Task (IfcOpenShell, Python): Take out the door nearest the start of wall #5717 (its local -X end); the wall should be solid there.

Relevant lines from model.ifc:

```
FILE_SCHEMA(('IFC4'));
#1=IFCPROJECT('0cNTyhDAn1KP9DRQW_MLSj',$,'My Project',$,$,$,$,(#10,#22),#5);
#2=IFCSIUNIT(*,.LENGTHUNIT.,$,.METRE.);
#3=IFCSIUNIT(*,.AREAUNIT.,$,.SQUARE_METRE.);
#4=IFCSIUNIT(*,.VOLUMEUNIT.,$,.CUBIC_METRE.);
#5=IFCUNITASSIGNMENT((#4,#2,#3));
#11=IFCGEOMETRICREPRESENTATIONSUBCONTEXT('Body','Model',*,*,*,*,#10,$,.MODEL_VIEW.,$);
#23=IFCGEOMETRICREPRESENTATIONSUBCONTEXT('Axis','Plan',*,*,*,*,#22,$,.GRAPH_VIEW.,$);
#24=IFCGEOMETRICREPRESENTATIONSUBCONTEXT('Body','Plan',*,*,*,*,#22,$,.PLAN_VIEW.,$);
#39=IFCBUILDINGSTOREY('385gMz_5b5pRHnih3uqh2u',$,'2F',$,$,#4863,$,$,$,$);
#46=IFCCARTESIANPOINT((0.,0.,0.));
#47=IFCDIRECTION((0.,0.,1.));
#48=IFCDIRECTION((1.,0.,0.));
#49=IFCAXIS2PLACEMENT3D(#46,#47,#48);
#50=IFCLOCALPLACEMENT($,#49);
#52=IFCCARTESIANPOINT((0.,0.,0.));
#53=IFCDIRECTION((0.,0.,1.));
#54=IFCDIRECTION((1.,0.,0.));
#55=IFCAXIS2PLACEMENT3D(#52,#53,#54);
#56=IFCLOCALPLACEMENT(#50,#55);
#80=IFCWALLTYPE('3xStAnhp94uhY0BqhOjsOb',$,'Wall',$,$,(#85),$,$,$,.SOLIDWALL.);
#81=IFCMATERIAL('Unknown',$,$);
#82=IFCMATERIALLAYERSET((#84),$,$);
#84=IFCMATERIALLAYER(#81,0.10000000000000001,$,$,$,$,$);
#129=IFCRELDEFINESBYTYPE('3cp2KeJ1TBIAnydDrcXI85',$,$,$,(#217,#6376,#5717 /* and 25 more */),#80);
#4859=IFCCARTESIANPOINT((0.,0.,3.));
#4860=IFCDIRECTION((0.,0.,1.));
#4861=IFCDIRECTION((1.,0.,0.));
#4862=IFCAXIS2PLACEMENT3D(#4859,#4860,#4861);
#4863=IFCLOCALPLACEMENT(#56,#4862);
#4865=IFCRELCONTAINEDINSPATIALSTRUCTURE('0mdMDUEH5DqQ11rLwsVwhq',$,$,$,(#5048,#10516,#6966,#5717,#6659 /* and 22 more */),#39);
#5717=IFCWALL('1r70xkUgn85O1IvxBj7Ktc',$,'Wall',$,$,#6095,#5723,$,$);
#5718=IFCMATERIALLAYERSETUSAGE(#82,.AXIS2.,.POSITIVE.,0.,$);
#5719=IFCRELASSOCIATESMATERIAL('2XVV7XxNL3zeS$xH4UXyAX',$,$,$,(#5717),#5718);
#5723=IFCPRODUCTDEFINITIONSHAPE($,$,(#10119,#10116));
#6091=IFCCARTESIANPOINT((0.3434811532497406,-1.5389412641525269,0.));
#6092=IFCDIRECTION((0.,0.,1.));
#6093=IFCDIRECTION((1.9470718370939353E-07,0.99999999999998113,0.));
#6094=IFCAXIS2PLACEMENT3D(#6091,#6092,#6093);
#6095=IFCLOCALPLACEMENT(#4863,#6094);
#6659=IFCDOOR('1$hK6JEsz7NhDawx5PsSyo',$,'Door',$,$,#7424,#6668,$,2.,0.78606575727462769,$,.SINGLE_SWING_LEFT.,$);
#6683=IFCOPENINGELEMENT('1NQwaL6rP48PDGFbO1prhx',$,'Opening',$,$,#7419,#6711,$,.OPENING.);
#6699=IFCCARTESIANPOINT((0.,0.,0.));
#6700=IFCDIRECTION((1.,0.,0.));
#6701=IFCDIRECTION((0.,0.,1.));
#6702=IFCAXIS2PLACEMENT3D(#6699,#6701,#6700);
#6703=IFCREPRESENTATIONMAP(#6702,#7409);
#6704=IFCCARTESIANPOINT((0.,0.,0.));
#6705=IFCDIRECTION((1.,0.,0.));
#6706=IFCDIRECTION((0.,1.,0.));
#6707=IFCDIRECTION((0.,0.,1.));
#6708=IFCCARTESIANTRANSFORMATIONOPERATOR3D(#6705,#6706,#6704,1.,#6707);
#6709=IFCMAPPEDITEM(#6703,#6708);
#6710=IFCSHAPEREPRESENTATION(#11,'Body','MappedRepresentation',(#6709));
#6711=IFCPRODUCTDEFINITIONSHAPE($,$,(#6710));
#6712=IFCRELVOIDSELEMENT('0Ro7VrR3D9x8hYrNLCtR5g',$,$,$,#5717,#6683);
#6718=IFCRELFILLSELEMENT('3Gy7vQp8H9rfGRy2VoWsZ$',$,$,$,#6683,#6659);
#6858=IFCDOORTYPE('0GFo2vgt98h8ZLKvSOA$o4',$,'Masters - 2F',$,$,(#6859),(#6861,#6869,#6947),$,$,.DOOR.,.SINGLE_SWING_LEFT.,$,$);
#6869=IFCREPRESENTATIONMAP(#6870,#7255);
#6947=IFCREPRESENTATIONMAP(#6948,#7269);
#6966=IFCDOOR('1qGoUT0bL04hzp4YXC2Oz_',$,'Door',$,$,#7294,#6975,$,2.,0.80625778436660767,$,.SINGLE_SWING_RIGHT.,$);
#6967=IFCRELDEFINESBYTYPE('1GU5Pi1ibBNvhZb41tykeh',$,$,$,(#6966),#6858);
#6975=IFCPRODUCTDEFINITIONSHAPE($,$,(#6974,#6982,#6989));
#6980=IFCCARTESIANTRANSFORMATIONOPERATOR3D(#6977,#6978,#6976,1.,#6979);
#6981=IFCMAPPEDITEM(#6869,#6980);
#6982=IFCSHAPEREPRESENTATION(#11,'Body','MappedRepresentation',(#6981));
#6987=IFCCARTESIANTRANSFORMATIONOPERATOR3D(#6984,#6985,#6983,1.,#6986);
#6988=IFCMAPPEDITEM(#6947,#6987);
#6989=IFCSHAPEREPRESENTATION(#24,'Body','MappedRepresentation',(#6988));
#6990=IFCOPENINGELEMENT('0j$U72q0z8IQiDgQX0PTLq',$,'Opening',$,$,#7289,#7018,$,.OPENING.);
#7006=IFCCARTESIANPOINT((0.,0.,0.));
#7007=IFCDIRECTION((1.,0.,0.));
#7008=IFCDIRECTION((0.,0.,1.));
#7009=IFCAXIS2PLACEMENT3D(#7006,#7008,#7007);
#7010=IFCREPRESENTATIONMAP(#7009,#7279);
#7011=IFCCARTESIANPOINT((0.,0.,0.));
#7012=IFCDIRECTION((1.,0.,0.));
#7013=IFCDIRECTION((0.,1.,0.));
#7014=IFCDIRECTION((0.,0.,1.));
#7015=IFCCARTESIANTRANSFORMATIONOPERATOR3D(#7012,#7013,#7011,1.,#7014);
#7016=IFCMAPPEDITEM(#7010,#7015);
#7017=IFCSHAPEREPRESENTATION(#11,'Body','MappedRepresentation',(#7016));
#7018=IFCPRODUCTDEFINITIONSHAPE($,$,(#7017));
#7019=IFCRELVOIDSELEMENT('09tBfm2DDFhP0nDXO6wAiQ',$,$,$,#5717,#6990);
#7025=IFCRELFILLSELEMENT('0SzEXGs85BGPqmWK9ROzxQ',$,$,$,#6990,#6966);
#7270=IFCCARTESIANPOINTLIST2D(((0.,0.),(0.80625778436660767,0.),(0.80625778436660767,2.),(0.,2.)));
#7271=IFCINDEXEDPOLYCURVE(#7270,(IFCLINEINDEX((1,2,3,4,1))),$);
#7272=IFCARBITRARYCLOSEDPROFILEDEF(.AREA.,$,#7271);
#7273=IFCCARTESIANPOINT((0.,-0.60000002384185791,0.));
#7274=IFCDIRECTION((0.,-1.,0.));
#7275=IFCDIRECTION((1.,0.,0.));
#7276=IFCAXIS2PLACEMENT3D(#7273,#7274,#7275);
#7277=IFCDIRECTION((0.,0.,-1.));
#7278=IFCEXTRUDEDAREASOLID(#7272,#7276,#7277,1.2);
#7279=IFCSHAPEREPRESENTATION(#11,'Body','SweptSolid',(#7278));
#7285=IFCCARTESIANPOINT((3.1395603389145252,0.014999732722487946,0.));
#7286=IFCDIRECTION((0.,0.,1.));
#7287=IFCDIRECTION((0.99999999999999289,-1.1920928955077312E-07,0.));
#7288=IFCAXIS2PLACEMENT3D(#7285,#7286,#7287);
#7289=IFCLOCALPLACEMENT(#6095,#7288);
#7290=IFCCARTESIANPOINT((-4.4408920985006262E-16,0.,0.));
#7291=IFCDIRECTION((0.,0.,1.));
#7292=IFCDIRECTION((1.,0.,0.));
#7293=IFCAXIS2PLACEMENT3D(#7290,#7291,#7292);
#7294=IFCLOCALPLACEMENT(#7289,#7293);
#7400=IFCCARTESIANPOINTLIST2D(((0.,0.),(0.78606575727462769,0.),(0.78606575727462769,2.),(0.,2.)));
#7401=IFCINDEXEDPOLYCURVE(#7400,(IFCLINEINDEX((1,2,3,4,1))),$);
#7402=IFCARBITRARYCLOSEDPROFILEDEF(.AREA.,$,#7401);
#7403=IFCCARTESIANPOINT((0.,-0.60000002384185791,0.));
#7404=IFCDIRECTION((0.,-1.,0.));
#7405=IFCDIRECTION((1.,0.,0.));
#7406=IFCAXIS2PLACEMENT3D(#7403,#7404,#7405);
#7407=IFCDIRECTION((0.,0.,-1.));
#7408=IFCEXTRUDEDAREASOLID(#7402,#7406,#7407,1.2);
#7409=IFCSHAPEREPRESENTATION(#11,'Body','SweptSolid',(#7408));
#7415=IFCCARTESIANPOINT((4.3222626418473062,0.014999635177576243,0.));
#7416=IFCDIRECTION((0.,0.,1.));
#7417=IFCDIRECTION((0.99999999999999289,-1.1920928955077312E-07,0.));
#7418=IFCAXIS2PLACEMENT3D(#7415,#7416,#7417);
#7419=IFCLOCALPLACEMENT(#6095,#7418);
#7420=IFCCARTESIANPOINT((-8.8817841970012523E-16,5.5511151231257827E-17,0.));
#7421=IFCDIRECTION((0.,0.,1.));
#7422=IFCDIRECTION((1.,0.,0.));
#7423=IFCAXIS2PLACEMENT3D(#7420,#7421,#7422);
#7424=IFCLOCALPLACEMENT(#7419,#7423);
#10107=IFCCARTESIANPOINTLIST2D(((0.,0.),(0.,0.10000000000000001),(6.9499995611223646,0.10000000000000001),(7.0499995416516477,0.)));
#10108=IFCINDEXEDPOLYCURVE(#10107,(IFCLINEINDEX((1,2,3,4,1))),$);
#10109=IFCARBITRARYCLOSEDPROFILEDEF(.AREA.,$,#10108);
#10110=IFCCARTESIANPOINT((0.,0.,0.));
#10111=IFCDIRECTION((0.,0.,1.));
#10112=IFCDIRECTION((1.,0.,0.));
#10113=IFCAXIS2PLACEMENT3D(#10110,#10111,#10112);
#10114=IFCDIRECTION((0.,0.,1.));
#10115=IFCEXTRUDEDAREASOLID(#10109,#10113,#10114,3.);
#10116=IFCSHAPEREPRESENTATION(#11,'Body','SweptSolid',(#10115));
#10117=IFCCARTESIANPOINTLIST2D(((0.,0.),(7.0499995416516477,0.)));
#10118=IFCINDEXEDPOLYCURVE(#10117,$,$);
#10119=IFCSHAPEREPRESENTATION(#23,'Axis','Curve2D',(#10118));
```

```python
import ifcopenshell
import ifcopenshell.api.feature
import ifcopenshell.api.root
import ifcopenshell.geom
import ifcopenshell.util.shape

model = ifcopenshell.open("model.ifc")
settings = ifcopenshell.geom.settings()


def volume(element):
    """Net volume in cubic metres, openings subtracted."""
    shape = ifcopenshell.geom.create_shape(settings, element)
    return ifcopenshell.util.shape.get_volume(shape.geometry)


door = model.by_id(6966)
opening = door.FillsVoids[0].RelatingOpeningElement
wall = opening.VoidsElements[0].RelatingBuildingElement
before = volume(wall)

ifcopenshell.api.root.remove_product(model, product=door)
ifcopenshell.api.feature.remove_feature(model, feature=opening)

after = volume(wall)

print(f"wall volume {before:.3f} -> {after:.3f} m3")

model.write("model_v2.ifc")
```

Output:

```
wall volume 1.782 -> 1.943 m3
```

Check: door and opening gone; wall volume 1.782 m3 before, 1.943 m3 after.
